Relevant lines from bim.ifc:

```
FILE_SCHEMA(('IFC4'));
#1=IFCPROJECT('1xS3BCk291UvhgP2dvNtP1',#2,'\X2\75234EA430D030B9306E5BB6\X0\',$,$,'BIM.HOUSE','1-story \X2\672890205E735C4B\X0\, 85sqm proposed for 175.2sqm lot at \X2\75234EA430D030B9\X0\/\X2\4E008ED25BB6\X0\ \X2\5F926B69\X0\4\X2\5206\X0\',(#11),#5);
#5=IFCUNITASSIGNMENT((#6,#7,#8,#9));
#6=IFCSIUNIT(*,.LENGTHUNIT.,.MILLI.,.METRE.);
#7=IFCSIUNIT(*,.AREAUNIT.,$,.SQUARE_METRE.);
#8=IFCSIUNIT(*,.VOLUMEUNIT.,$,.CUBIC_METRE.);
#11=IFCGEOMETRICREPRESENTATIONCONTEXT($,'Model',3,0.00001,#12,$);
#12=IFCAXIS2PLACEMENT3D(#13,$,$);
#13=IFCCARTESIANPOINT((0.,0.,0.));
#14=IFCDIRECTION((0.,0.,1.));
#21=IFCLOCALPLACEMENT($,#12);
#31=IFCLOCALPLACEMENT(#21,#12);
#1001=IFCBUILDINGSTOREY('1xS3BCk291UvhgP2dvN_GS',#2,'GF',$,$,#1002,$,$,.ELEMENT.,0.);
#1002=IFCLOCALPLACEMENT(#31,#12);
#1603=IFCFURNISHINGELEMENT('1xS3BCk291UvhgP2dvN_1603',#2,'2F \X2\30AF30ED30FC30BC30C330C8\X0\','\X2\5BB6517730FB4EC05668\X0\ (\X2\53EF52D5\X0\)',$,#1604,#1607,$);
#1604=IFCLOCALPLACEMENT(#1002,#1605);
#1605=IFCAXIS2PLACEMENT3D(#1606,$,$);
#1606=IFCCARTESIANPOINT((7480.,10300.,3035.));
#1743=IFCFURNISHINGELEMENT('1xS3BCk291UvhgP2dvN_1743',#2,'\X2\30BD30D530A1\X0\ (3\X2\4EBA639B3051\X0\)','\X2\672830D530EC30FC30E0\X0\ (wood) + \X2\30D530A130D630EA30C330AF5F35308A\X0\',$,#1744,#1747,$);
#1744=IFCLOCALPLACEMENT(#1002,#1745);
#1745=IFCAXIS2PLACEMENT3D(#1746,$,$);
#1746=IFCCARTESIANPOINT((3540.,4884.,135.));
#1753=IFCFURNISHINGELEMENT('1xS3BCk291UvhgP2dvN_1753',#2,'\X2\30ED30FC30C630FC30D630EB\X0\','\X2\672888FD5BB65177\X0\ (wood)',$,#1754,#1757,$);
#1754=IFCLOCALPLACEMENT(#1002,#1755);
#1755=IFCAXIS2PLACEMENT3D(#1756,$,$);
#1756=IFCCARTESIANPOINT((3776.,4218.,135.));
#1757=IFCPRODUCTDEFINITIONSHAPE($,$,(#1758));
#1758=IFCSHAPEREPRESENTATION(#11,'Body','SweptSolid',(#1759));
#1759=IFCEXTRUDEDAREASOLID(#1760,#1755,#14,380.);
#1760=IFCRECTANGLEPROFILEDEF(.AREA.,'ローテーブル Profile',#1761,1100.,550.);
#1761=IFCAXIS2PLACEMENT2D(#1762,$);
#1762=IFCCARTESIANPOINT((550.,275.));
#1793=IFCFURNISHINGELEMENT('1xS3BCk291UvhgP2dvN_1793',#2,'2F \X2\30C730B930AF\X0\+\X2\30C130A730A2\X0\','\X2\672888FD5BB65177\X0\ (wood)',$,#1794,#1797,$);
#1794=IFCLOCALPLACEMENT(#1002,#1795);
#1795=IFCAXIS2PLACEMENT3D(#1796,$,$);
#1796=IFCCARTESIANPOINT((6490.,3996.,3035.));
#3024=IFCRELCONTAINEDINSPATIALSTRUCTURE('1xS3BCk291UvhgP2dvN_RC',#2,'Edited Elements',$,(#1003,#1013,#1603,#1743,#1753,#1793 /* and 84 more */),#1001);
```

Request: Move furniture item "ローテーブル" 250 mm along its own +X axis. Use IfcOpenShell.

```python
import ifcopenshell
import ifcopenshell.api.geometry
import ifcopenshell.util.placement
import ifcopenshell.util.unit

model = ifcopenshell.open("bim.ifc")
unit_scale = ifcopenshell.util.unit.calculate_unit_scale(model)

item = model.by_id(1753)
matrix = ifcopenshell.util.placement.get_local_placement(item.ObjectPlacement)
matrix[:3, 3] += matrix[:3, 0] * 0.25 / unit_scale
ifcopenshell.api.geometry.edit_object_placement(model, product=item, matrix=matrix, is_si=False)

print(ifcopenshell.util.placement.get_local_placement(item.ObjectPlacement).round(3) + 0.0)

model.write("bim_edited.ifc")
```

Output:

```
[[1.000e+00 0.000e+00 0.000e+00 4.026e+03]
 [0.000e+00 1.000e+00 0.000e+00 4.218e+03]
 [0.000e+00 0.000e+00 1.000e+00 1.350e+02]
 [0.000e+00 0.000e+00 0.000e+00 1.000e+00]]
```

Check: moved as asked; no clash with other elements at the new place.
